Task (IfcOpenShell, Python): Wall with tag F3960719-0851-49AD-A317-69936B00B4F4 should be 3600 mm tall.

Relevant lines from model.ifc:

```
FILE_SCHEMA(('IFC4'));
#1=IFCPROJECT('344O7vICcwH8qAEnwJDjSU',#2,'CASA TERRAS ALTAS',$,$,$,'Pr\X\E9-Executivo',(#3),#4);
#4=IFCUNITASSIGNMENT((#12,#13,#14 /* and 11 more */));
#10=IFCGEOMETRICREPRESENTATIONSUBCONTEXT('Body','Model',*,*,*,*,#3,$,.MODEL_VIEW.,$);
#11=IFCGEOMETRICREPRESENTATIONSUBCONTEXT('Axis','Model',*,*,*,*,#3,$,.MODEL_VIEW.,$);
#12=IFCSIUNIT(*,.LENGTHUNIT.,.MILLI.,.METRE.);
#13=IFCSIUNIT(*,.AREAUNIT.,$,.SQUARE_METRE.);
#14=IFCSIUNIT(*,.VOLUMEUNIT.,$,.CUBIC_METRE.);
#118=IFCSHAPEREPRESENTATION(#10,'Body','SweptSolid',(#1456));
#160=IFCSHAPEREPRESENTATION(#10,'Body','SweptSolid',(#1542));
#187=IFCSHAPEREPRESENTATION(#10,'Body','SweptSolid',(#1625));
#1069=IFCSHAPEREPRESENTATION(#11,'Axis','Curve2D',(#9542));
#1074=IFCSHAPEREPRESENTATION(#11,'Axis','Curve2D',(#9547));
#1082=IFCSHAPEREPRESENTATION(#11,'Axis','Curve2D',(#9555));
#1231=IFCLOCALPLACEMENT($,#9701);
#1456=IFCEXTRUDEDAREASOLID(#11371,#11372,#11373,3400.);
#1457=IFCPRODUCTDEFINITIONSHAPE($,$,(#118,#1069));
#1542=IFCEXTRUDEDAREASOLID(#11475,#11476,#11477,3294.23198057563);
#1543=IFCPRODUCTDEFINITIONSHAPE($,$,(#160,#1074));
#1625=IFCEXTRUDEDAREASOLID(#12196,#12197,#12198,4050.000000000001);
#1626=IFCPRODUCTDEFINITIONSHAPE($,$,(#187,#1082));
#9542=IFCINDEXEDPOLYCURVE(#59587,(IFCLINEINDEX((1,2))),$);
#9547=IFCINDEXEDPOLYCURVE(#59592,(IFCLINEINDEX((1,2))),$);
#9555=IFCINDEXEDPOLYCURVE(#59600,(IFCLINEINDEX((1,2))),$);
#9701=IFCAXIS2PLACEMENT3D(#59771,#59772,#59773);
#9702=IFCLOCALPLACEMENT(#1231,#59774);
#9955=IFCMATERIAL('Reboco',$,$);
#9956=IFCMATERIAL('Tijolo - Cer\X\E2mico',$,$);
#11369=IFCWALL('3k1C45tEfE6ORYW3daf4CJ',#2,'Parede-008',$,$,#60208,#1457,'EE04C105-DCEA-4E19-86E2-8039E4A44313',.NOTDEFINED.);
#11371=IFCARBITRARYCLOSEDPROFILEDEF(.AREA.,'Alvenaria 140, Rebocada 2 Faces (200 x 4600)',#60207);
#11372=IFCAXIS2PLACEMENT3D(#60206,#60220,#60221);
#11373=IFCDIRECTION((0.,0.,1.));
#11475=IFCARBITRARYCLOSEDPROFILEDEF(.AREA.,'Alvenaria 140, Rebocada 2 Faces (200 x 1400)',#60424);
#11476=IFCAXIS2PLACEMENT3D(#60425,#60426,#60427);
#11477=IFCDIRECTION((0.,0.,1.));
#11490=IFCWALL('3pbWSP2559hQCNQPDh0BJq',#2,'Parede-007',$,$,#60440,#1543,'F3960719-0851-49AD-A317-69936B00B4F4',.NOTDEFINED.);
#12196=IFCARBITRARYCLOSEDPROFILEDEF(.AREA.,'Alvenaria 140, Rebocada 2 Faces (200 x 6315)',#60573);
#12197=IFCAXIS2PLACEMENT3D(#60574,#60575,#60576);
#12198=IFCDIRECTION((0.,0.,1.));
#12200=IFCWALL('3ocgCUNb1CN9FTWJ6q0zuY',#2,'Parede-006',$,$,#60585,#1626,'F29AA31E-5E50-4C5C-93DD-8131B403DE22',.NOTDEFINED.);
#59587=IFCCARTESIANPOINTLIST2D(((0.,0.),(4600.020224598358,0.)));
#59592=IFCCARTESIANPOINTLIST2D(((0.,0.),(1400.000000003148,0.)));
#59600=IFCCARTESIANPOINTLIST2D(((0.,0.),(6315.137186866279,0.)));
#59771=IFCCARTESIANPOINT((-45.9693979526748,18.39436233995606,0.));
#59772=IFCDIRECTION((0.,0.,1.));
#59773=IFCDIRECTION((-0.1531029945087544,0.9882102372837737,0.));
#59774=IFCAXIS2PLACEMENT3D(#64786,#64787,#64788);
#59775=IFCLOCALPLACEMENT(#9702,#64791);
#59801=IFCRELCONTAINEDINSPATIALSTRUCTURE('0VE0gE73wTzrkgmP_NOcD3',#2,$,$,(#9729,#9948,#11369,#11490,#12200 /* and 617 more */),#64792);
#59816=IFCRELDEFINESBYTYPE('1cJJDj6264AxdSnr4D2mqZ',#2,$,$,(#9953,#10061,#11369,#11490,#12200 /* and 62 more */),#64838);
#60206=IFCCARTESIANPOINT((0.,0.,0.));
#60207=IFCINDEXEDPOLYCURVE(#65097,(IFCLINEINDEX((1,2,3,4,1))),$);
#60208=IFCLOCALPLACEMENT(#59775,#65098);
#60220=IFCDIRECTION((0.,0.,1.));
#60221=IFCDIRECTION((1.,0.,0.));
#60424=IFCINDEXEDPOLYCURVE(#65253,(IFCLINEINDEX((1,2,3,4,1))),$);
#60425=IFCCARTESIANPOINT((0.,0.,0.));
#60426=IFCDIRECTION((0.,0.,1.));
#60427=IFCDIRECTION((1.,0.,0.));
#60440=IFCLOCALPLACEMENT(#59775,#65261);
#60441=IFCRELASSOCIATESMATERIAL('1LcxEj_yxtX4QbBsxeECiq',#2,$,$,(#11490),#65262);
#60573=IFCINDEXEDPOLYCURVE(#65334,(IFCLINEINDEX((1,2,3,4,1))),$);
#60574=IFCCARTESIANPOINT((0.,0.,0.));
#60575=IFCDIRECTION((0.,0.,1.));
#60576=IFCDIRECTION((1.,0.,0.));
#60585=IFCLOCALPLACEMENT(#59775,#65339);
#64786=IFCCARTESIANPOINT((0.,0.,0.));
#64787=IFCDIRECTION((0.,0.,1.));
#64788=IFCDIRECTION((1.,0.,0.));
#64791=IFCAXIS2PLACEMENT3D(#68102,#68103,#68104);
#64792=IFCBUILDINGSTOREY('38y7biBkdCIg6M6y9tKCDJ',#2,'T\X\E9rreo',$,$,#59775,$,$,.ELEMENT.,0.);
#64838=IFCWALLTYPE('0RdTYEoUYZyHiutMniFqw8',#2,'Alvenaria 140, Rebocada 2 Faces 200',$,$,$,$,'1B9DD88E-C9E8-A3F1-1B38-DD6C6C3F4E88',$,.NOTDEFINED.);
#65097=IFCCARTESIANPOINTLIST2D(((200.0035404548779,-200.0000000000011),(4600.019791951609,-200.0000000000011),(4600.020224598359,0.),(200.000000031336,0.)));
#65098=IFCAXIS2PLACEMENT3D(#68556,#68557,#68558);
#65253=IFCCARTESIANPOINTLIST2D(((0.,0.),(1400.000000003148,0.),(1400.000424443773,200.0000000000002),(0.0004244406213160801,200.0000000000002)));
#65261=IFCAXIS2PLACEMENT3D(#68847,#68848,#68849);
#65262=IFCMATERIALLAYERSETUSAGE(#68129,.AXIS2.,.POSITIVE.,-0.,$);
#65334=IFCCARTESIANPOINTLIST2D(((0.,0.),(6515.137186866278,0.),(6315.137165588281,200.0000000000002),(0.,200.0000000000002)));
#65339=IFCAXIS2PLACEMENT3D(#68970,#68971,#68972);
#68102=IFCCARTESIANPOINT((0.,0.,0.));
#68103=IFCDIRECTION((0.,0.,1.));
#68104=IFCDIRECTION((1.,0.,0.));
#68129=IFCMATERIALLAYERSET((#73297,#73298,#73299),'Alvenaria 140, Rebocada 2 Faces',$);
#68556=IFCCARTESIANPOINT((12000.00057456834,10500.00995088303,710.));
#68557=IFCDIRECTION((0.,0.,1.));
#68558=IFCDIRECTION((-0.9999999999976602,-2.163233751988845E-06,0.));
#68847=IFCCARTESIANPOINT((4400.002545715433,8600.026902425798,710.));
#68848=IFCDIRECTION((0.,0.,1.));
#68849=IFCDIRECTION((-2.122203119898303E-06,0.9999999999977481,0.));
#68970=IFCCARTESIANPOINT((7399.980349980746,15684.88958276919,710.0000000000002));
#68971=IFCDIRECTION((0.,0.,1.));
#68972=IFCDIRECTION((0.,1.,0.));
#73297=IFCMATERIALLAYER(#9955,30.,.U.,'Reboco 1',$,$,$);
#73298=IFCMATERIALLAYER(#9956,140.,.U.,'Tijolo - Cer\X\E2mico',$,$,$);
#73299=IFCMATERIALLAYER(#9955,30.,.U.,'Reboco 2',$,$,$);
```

```python
import ifcopenshell
import ifcopenshell.geom
import ifcopenshell.util.representation
import ifcopenshell.util.shape
import ifcopenshell.util.unit

model = ifcopenshell.open("model.ifc")
unit_scale = ifcopenshell.util.unit.calculate_unit_scale(model)
settings = ifcopenshell.geom.settings()


def volume(element):
    """Net volume in cubic metres, openings subtracted."""
    shape = ifcopenshell.geom.create_shape(settings, element)
    return ifcopenshell.util.shape.get_volume(shape.geometry)


wall = model.by_guid("3pbWSP2559hQCNQPDh0BJq")
before = volume(wall)

body = ifcopenshell.util.representation.get_representation(wall, "Model", "Body")
solid = body.Items[0]
old_height = solid.Depth
solid.Depth = 3.6 / unit_scale
after = volume(wall)

print(f"height {old_height:g} -> {solid.Depth:g}, volume {before:.3f} -> {after:.3f} m3")

model.write("model-out.ifc")
```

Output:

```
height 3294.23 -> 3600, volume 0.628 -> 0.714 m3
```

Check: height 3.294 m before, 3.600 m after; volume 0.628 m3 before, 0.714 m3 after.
